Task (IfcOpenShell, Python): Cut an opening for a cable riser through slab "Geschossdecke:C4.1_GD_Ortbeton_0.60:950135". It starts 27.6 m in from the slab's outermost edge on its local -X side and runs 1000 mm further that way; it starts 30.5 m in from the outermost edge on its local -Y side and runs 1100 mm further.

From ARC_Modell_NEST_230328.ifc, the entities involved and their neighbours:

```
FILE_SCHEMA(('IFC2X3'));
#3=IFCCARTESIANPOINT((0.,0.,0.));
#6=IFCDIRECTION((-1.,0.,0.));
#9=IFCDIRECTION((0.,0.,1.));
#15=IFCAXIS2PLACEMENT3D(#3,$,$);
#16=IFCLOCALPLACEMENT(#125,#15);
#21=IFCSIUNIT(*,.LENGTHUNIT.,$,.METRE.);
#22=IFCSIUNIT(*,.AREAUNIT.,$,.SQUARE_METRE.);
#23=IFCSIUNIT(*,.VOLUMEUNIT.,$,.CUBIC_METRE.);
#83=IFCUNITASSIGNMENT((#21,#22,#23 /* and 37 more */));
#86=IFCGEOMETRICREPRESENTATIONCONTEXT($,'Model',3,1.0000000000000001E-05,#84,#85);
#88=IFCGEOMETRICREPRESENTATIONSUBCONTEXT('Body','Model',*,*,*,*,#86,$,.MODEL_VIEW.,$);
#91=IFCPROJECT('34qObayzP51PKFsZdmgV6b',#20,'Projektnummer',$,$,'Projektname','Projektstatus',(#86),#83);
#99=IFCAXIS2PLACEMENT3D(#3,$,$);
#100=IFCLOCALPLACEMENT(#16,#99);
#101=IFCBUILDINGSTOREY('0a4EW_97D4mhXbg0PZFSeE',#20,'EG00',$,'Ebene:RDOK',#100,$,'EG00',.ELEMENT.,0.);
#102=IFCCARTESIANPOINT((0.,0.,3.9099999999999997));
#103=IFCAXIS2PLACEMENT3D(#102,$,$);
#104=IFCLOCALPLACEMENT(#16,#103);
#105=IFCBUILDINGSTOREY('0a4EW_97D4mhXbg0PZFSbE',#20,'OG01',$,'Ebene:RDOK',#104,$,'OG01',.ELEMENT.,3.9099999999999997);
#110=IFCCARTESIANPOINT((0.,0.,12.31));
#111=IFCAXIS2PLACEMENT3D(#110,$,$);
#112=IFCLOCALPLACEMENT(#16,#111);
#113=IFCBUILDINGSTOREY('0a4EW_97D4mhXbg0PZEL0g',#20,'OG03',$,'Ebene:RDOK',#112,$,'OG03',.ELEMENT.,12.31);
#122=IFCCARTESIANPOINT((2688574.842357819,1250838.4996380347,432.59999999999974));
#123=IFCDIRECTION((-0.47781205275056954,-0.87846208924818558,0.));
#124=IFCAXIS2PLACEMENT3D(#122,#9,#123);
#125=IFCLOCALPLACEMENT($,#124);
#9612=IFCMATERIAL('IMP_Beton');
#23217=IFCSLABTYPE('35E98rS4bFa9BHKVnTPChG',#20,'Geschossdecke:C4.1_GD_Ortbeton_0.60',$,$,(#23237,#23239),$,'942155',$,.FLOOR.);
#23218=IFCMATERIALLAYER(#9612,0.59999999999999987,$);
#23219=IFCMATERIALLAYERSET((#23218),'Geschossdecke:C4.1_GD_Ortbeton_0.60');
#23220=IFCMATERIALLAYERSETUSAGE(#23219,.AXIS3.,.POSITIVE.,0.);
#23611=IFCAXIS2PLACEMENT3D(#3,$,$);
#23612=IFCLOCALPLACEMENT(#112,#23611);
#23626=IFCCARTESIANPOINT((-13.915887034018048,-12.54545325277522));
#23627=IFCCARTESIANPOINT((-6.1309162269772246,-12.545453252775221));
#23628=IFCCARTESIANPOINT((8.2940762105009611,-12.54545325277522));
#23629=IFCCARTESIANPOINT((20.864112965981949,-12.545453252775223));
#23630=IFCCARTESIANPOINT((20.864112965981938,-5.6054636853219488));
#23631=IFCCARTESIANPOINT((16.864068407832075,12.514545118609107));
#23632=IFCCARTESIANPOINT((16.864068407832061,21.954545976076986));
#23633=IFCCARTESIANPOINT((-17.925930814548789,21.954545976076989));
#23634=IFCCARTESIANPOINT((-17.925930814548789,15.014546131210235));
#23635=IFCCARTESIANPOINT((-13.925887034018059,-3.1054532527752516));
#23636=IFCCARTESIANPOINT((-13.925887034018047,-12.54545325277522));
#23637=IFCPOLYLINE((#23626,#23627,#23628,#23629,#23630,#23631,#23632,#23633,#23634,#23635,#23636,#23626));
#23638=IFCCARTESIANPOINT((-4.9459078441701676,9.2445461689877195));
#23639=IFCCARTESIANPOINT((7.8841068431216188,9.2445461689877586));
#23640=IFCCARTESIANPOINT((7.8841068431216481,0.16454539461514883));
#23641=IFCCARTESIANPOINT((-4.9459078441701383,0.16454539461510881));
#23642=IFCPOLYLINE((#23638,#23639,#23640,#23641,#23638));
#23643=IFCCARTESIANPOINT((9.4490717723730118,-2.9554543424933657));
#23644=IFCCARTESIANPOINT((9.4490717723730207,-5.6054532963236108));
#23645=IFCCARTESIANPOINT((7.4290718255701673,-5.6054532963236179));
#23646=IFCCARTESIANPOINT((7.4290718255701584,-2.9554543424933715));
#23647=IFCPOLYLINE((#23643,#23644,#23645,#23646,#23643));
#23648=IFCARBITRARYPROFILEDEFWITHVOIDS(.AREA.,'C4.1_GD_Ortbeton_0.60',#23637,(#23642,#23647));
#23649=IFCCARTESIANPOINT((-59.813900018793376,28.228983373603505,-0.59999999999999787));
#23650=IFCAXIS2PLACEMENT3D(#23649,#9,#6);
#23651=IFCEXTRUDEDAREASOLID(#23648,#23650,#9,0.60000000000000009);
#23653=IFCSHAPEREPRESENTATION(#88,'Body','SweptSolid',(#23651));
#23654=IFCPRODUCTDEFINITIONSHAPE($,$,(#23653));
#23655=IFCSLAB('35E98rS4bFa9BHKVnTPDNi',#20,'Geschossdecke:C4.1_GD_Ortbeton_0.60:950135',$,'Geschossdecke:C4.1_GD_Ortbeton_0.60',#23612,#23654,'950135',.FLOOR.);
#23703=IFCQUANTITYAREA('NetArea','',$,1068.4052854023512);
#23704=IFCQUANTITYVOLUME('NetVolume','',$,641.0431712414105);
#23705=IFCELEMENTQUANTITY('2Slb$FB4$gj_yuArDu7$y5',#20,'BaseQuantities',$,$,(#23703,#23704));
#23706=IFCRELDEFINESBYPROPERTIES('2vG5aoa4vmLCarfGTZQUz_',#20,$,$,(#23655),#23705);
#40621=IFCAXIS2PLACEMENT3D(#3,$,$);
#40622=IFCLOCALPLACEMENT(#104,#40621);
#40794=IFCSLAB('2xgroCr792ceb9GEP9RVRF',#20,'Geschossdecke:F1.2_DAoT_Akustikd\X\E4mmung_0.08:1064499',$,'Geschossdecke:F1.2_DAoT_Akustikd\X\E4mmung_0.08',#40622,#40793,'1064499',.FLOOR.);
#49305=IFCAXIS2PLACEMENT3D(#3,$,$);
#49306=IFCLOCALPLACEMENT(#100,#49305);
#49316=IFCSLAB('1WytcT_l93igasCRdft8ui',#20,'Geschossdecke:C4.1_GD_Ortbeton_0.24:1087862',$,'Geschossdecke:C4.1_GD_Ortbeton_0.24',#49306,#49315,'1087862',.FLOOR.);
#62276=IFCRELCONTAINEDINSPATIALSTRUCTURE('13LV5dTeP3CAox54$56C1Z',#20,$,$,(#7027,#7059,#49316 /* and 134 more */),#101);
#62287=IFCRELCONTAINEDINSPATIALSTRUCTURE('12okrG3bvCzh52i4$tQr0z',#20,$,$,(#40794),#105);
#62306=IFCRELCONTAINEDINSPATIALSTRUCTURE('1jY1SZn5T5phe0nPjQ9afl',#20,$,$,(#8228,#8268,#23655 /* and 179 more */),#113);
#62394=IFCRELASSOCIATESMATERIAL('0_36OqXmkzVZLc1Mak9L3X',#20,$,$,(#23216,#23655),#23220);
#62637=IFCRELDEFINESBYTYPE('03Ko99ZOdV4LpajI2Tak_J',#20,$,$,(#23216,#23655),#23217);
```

```python
import numpy as np
import ifcopenshell
import ifcopenshell.api.feature
import ifcopenshell.api.geometry
import ifcopenshell.api.pset
import ifcopenshell.api.root
import ifcopenshell.geom
import ifcopenshell.util.element
import ifcopenshell.util.placement
import ifcopenshell.util.representation
import ifcopenshell.util.shape
import ifcopenshell.util.unit

model = ifcopenshell.open("ARC_Modell_NEST_230328.ifc")
unit_scale = ifcopenshell.util.unit.calculate_unit_scale(model)
area_scale = ifcopenshell.util.unit.calculate_unit_scale(model, "AREAUNIT")
volume_scale = ifcopenshell.util.unit.calculate_unit_scale(model, "VOLUMEUNIT")
settings = ifcopenshell.geom.settings()


def volume(element):
    """Net volume in cubic metres, openings subtracted."""
    shape = ifcopenshell.geom.create_shape(settings, element)
    return ifcopenshell.util.shape.get_volume(shape.geometry)


slab = model.by_id(23655)
before = volume(slab)

# Extent in the slab's own axes, in metres. The edges named are its -X and -Y sides.
slab_shape = ifcopenshell.geom.create_shape(settings, slab)
vertices = ifcopenshell.util.shape.get_vertices(slab_shape.geometry)
x_min, y_min, bottom = vertices.min(axis=0)
top = vertices[:, 2].max()

opening = ifcopenshell.api.root.create_entity(model, ifc_class="IfcOpeningElement", name="Cable riser opening")
context = ifcopenshell.util.representation.get_context(model, "Model", "Body", "MODEL_VIEW")
width, depth = 1, 1.1
outline = [(0.0, 0.0), (width, 0.0), (width, depth), (0.0, depth), (0.0, 0.0)]
# Overshoot both faces by 50 mm so the cut is clean.
shape = ifcopenshell.api.geometry.add_slab_representation(
    model, context=context, depth=top - bottom + 0.1, polyline=outline
)
ifcopenshell.api.geometry.assign_representation(model, product=opening, representation=shape)

matrix = ifcopenshell.util.placement.get_local_placement(slab.ObjectPlacement)
matrix[:, 3] = matrix @ np.append(np.array([x_min + 27.6, y_min + 30.5, bottom - 0.05]) / unit_scale, 1.0)
ifcopenshell.api.geometry.edit_object_placement(model, product=opening, matrix=matrix, is_si=False)
ifcopenshell.api.feature.add_feature(model, feature=opening, element=slab)

after = volume(slab)

# Update the slab's stored quantities.
qto = model.by_id(ifcopenshell.util.element.get_pset(slab, "BaseQuantities", should_inherit=False)["id"])
ifcopenshell.api.pset.edit_qto(model, qto=qto, properties={
    "NetArea": after / (top - bottom) / area_scale,
    "NetVolume": after / volume_scale,
})

print(f"slab volume {before:.3f} -> {after:.3f} m3")

model.write("ARC_Modell_NEST_230328_v2.ifc")
```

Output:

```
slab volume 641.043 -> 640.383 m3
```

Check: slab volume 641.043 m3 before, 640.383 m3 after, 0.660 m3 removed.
